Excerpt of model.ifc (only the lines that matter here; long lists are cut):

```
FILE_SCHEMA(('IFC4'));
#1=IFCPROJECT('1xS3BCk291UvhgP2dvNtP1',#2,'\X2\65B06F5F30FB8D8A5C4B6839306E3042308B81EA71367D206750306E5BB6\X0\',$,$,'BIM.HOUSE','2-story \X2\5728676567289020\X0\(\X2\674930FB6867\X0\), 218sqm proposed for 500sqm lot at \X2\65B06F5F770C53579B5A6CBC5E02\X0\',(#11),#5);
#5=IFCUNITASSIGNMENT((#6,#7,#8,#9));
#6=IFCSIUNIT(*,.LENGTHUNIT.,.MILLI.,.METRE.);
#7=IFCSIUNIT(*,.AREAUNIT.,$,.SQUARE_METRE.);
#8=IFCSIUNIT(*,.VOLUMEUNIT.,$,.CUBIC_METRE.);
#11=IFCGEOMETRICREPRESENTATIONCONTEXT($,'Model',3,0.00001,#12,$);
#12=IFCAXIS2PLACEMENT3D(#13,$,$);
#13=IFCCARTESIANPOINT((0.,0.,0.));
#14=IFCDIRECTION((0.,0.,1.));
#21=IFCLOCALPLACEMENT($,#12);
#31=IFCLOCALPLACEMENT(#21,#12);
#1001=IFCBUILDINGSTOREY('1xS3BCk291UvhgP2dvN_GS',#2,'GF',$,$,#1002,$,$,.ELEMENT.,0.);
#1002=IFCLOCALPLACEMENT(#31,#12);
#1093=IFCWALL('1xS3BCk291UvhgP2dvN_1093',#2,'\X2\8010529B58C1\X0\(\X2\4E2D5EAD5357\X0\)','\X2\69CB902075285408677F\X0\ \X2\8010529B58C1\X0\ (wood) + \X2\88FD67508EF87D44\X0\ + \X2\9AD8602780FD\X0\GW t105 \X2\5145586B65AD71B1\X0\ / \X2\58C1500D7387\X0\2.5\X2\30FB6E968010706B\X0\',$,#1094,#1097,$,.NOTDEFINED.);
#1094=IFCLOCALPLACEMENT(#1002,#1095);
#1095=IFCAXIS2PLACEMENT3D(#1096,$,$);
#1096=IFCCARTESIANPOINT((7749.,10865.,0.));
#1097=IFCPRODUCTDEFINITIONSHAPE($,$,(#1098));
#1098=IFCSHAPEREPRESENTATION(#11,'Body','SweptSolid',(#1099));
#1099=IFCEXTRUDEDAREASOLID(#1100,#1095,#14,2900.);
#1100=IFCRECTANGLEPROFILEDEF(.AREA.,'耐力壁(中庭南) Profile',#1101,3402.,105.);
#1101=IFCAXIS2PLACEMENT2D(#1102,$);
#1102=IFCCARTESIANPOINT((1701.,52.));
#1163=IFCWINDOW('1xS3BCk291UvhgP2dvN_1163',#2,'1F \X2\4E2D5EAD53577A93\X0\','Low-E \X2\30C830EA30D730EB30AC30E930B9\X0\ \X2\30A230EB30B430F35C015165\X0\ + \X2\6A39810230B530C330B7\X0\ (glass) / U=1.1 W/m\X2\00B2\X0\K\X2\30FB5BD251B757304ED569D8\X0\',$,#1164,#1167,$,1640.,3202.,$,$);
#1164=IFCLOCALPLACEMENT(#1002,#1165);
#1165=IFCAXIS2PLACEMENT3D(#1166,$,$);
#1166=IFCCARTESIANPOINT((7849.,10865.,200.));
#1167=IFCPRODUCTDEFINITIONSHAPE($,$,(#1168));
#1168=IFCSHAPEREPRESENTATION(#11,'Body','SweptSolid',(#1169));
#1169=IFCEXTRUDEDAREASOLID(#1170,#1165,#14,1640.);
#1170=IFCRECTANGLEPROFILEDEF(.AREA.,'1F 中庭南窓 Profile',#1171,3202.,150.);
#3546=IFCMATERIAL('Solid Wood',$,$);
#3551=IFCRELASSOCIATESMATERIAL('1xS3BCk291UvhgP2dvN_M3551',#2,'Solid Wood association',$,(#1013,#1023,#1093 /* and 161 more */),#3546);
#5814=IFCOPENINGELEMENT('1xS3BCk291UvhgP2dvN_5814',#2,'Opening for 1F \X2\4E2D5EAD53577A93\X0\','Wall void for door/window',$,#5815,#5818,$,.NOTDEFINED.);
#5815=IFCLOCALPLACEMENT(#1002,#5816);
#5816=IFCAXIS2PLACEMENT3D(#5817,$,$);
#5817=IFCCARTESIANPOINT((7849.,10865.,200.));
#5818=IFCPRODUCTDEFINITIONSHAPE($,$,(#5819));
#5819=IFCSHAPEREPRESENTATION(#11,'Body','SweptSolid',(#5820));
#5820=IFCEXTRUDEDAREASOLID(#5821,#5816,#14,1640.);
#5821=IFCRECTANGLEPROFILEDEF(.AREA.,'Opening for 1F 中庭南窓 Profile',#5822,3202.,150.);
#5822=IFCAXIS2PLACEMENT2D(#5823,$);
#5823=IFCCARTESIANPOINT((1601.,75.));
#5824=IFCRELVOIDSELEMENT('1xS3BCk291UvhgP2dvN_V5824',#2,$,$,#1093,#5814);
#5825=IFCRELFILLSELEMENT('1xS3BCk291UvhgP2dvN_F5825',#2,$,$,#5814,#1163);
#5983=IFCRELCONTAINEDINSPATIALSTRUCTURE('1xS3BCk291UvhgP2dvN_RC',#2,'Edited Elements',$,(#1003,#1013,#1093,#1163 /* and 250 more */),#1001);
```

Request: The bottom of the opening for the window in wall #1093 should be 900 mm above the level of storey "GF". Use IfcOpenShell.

```python
import numpy as np
import ifcopenshell
import ifcopenshell.api.geometry
import ifcopenshell.geom
import ifcopenshell.util.element
import ifcopenshell.util.placement
import ifcopenshell.util.shape
import ifcopenshell.util.unit

model = ifcopenshell.open("model.ifc")
unit_scale = ifcopenshell.util.unit.calculate_unit_scale(model)

window = model.by_guid("1xS3BCk291UvhgP2dvN_1163")
opening = window.FillsVoids[0].RelatingOpeningElement
storey = ifcopenshell.util.element.get_container(window, ifc_class="IfcBuildingStorey")
level = ifcopenshell.util.placement.get_local_placement(storey.ObjectPlacement)[2, 3]

# The opening's origin need not be at the sill, so measure its lowest point.
shape = ifcopenshell.geom.create_shape(ifcopenshell.geom.settings(), opening)
bottom = ifcopenshell.util.shape.get_shape_bottom_elevation(shape, shape.geometry) / unit_scale
dz = level + 900.0 - bottom

shift = np.array([0.0, 0.0, dz])
# The window is not placed relative to its opening, so move both.
for product in (opening, window):
    matrix = ifcopenshell.util.placement.get_local_placement(product.ObjectPlacement)
    matrix[:3, 3] += shift
    ifcopenshell.api.geometry.edit_object_placement(model, product=product, matrix=matrix, is_si=False)

print(f"moved by {dz * unit_scale:+.3f} m")

model.write("model_updated.ifc")
```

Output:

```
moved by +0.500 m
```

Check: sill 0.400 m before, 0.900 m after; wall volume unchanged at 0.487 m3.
